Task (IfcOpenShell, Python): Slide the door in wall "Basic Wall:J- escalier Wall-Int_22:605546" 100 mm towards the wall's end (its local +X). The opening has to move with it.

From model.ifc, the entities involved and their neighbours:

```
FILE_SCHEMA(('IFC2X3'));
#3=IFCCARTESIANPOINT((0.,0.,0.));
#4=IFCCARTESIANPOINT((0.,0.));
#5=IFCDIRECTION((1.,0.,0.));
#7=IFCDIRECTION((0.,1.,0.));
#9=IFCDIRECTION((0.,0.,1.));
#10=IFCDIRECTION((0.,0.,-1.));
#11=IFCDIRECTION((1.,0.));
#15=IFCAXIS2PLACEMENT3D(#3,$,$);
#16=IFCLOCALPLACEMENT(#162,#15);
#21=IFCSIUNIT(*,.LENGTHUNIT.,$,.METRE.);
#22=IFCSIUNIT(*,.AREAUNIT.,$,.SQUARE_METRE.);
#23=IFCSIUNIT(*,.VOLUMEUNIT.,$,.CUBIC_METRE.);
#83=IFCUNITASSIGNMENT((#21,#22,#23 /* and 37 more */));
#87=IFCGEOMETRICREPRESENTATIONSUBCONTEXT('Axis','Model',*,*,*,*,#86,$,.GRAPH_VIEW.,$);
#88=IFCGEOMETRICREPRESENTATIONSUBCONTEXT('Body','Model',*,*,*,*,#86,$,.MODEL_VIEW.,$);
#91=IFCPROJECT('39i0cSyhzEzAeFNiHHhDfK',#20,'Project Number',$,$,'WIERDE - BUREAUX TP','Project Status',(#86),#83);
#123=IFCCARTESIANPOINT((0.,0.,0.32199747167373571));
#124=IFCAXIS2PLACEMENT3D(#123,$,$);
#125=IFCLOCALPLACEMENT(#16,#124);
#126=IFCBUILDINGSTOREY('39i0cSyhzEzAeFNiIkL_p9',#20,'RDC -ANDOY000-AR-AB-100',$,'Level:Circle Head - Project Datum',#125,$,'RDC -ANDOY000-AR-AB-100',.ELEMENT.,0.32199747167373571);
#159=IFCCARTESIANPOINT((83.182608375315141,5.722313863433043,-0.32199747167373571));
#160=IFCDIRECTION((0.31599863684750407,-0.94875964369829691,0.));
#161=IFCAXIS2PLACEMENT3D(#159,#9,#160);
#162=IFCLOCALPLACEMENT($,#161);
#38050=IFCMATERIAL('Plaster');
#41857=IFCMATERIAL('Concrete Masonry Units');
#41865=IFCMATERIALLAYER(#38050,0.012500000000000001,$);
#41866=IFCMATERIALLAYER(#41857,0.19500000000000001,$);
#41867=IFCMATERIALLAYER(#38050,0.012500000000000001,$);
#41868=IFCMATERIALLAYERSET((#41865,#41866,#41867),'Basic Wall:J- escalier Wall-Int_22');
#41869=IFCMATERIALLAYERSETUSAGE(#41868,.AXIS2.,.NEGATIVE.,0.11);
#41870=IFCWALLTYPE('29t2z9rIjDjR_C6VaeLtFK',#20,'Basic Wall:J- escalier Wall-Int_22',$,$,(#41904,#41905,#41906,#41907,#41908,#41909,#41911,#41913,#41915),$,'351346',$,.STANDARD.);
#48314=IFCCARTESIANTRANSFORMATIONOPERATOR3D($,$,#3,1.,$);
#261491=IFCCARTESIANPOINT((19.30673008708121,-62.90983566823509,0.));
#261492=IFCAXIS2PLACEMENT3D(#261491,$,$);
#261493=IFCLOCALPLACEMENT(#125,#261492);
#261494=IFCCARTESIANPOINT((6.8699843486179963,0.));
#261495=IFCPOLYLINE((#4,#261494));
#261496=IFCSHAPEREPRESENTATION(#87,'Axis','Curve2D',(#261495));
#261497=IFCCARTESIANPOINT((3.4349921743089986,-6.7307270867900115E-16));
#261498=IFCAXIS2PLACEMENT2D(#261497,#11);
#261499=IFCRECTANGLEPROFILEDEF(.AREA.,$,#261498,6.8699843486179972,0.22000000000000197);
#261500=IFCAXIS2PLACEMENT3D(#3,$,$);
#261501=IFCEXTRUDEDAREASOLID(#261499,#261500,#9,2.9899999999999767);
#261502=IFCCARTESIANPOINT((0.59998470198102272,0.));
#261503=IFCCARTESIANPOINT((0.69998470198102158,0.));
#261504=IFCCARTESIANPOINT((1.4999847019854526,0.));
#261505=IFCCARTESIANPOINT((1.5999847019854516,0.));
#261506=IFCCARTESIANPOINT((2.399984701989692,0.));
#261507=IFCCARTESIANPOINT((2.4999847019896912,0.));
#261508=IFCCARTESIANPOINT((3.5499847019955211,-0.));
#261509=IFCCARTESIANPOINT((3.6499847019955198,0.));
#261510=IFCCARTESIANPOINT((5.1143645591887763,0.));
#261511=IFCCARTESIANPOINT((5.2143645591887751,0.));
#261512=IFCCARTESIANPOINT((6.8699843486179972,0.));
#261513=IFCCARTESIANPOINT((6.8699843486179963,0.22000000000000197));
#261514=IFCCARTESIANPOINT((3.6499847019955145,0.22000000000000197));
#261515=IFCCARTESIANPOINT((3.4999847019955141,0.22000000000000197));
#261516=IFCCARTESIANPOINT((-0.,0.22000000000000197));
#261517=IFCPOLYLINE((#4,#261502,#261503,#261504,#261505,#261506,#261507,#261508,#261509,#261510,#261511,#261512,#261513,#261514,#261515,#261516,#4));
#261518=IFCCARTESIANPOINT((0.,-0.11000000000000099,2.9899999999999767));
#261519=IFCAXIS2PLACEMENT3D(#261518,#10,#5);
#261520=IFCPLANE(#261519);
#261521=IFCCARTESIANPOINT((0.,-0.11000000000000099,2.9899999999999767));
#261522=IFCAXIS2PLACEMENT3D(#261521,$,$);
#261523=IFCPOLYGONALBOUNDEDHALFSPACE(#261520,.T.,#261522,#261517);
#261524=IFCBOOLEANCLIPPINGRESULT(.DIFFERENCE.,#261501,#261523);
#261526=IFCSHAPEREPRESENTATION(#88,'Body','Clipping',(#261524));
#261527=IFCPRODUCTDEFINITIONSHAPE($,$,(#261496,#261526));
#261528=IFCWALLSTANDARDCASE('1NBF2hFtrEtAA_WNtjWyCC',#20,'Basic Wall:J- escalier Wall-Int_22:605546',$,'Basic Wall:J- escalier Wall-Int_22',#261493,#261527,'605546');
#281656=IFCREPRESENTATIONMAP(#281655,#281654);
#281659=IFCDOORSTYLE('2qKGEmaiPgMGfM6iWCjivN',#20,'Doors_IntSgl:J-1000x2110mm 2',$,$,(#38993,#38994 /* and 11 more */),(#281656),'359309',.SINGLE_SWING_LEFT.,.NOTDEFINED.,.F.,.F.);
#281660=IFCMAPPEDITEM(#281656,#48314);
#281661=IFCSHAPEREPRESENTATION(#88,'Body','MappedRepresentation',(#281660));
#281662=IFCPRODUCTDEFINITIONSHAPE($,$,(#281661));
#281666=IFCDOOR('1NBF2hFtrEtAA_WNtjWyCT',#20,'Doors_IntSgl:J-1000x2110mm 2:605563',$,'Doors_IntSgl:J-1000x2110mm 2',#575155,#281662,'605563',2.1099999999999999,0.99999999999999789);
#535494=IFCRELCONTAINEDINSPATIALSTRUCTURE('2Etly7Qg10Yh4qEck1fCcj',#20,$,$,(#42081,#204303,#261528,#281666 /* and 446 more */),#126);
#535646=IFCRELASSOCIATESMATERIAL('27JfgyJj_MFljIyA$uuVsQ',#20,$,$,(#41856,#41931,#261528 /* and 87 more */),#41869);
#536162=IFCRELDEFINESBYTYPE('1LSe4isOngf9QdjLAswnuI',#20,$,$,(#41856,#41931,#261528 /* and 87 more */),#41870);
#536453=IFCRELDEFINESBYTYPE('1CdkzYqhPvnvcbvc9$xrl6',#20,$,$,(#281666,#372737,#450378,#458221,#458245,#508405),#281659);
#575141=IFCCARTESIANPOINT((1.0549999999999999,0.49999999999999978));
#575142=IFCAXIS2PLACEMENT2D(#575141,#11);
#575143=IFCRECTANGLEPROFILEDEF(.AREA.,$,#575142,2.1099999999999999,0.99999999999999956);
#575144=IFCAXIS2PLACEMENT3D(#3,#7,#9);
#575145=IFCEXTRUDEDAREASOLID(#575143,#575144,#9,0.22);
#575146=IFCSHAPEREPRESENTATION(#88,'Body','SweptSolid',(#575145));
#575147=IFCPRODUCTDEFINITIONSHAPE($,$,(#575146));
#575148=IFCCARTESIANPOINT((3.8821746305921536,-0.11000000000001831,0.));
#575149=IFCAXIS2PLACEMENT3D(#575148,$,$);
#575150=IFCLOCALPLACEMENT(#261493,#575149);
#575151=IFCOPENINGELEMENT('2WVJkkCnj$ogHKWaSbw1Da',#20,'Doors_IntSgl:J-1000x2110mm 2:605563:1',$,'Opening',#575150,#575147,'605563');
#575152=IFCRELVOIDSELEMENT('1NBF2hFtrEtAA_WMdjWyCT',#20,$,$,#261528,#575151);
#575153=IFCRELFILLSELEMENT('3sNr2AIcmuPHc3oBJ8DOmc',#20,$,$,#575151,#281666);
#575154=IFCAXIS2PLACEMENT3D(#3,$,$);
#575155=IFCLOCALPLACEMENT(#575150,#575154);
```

```python
import ifcopenshell
import ifcopenshell.api.geometry
import ifcopenshell.util.placement

model = ifcopenshell.open("model.ifc")

door = model.by_guid("1NBF2hFtrEtAA_WNtjWyCT")
opening = door.FillsVoids[0].RelatingOpeningElement
wall = opening.VoidsElements[0].RelatingBuildingElement

wall_matrix = ifcopenshell.util.placement.get_local_placement(wall.ObjectPlacement)
shift = wall_matrix[:3, 0] * 0.1
before = ifcopenshell.util.placement.get_local_placement(door.ObjectPlacement)[:3, 3].copy()

# The door is placed relative to its opening, so it follows when the opening moves.
matrix = ifcopenshell.util.placement.get_local_placement(opening.ObjectPlacement)
matrix[:3, 3] += shift
ifcopenshell.api.geometry.edit_object_placement(
    model, product=opening, matrix=matrix, is_si=False, should_transform_children=True
)

after = ifcopenshell.util.placement.get_local_placement(door.ObjectPlacement)[:3, 3]
print("door moved by", (after - before).round(3) + 0.0)

model.write("model_updated.ifc")
```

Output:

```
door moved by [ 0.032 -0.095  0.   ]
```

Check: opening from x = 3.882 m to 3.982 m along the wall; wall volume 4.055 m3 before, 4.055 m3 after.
